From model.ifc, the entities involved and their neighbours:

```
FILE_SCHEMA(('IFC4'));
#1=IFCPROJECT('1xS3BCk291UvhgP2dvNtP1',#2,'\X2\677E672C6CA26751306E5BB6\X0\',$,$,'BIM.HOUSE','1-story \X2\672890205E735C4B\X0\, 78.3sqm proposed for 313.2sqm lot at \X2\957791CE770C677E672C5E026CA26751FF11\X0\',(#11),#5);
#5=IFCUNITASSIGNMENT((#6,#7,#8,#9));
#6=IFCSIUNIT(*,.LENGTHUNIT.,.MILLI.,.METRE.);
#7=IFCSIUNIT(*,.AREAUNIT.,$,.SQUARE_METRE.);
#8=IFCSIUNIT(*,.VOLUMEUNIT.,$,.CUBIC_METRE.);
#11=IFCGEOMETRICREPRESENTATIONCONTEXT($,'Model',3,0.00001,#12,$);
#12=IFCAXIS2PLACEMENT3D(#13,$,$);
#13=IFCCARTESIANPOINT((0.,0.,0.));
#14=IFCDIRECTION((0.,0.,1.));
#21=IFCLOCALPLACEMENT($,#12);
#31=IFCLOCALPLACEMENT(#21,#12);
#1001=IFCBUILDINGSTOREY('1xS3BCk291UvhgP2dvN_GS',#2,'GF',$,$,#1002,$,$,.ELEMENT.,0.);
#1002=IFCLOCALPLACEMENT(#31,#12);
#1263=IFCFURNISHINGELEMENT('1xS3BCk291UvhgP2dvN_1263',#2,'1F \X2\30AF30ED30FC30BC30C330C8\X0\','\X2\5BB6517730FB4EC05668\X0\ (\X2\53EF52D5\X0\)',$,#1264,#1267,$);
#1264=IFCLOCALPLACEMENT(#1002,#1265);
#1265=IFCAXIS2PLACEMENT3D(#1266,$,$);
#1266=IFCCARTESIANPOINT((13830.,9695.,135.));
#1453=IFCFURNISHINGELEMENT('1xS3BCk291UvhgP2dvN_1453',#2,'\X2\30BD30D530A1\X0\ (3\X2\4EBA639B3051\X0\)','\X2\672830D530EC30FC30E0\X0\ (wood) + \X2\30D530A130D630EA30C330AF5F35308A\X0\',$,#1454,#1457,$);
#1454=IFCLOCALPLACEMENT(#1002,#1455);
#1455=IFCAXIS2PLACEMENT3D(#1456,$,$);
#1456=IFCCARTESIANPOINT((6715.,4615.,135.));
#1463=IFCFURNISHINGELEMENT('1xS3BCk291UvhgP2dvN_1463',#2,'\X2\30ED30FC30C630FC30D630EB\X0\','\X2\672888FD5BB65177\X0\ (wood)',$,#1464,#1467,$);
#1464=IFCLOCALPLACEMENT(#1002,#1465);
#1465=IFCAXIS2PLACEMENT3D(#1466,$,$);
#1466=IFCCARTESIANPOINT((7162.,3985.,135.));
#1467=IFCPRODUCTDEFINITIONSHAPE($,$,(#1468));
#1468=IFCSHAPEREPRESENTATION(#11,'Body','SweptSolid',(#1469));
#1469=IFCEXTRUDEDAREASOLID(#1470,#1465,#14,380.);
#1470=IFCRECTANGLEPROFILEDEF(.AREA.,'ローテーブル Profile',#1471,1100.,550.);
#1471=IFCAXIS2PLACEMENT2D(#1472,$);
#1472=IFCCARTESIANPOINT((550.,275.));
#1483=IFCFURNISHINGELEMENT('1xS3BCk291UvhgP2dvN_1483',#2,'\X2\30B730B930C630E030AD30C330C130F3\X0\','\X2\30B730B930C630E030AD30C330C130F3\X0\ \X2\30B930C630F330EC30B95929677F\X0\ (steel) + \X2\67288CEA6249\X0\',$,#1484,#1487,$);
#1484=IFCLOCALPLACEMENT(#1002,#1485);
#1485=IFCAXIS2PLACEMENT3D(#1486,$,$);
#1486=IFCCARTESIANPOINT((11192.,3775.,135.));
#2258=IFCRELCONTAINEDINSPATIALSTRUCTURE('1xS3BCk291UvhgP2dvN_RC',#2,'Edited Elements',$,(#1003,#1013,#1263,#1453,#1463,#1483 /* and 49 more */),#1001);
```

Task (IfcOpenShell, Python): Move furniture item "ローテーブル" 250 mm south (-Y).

```python
import ifcopenshell
import ifcopenshell.api.geometry
import ifcopenshell.util.placement
import ifcopenshell.util.unit

model = ifcopenshell.open("model.ifc")
unit_scale = ifcopenshell.util.unit.calculate_unit_scale(model)

item = model.by_id(1463)
matrix = ifcopenshell.util.placement.get_local_placement(item.ObjectPlacement)
matrix[1, 3] -= 0.25 / unit_scale
ifcopenshell.api.geometry.edit_object_placement(model, product=item, matrix=matrix, is_si=False)

print(ifcopenshell.util.placement.get_local_placement(item.ObjectPlacement).round(3) + 0.0)

model.write("model_edited.ifc")
```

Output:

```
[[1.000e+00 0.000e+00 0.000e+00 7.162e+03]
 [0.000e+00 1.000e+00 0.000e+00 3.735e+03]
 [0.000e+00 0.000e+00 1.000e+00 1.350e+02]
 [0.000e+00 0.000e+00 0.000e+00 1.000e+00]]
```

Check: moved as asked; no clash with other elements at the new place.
